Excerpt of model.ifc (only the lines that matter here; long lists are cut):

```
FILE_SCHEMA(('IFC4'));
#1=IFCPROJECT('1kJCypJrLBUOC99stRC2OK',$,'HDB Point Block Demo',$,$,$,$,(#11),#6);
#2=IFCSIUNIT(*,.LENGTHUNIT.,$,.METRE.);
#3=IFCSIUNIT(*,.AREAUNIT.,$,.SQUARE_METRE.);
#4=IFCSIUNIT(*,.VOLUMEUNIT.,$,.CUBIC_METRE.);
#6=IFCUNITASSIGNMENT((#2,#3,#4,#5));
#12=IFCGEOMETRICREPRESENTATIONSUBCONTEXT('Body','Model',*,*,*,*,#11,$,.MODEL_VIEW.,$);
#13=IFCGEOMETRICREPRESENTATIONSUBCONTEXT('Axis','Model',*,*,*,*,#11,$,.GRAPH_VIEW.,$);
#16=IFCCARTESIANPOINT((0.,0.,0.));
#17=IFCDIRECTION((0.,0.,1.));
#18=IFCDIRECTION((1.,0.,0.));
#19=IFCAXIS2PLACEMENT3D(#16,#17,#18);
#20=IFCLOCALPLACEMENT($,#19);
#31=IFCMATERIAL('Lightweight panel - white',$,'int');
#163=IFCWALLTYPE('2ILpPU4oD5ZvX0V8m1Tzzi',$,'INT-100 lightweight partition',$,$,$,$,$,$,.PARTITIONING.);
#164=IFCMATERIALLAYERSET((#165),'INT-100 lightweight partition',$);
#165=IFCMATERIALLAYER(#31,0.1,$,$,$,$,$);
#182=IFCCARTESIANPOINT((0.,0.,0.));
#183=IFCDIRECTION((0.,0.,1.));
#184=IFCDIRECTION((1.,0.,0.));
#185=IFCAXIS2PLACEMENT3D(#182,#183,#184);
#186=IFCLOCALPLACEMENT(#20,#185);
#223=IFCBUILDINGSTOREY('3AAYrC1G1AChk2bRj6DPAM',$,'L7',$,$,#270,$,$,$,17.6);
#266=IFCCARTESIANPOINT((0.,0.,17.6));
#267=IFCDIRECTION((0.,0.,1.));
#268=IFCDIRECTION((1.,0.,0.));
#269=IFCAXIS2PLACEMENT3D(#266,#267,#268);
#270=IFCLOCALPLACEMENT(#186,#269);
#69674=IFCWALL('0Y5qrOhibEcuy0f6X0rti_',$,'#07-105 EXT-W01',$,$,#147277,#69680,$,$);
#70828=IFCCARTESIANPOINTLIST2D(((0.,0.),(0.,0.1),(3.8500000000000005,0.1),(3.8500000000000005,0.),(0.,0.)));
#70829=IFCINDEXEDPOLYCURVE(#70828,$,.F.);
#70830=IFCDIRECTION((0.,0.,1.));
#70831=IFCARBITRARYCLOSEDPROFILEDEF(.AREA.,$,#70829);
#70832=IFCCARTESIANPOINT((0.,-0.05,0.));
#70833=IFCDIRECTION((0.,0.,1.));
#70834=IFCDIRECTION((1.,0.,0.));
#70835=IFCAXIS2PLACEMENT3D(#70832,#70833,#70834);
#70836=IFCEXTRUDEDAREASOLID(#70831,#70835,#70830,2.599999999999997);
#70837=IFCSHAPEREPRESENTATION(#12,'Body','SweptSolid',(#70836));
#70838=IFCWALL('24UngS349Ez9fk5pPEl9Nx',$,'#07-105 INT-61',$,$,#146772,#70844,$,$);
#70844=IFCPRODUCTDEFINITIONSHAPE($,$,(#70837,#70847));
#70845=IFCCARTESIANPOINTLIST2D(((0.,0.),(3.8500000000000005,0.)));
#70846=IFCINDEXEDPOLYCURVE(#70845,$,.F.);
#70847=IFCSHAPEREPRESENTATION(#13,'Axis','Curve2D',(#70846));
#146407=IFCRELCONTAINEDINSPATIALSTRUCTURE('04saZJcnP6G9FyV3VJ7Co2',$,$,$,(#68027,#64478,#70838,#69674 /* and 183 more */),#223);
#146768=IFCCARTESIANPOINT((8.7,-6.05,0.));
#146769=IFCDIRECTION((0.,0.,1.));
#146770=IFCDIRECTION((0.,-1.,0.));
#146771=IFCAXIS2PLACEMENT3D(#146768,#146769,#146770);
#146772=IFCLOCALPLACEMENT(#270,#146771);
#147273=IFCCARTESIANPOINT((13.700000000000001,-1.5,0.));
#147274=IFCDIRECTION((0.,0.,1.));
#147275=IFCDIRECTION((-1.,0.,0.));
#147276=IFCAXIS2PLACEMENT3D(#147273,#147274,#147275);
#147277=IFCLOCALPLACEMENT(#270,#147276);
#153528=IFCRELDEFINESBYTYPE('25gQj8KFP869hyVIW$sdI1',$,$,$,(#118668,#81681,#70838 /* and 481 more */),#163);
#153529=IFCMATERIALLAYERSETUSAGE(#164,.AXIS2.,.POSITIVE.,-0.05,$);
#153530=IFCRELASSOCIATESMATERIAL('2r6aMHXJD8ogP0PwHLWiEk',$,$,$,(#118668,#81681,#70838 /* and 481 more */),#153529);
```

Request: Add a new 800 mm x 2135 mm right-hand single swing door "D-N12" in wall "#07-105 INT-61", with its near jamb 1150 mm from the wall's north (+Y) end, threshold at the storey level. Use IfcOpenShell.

```python
import numpy as np
import ifcopenshell
import ifcopenshell.api.feature
import ifcopenshell.api.geometry
import ifcopenshell.api.root
import ifcopenshell.api.spatial
import ifcopenshell.geom
import ifcopenshell.util.element
import ifcopenshell.util.placement
import ifcopenshell.util.representation
import ifcopenshell.util.shape
import ifcopenshell.util.unit

model = ifcopenshell.open("model.ifc")
unit_scale = ifcopenshell.util.unit.calculate_unit_scale(model)
settings = ifcopenshell.geom.settings()


def volume(element):
    """Net volume in cubic metres, openings subtracted."""
    shape = ifcopenshell.geom.create_shape(settings, element)
    return ifcopenshell.util.shape.get_volume(shape.geometry)


wall = model.by_guid("24UngS349Ez9fk5pPEl9Nx")
storey = ifcopenshell.util.element.get_container(wall, ifc_class="IfcBuildingStorey")
context = ifcopenshell.util.representation.get_context(model, "Model", "Body", "MODEL_VIEW")
before = volume(wall)

width, height, from_end, sill = 0.8, 2.135, 1.15, 0.0  # metres

# The wall runs along its own X axis, and the end named is its -X end.
wall_shape = ifcopenshell.geom.create_shape(settings, wall)
x, y, z = ifcopenshell.util.shape.get_vertices(wall_shape.geometry).T
start = x.min() + from_end
face, thickness = float(y.min()), float(y.max() - y.min())
wall_matrix = ifcopenshell.util.placement.get_local_placement(wall.ObjectPlacement)
level = ifcopenshell.util.placement.get_local_placement(storey.ObjectPlacement)[2, 3]


def in_wall(x, y):
    """Placement at x, y metres in the wall's axes, at sill height."""
    matrix = wall_matrix.copy()
    matrix[:, 3] = wall_matrix @ np.array([x / unit_scale, y / unit_scale, 0.0, 1.0])
    matrix[2, 3] = level + sill / unit_scale
    return matrix


# Opening: a box that overshoots both wall faces by 50 mm.
opening = ifcopenshell.api.root.create_entity(model, ifc_class="IfcOpeningElement", predefined_type="OPENING")
box = ifcopenshell.api.geometry.add_wall_representation(
    model, context=context, length=width, height=height, thickness=thickness + 0.1
)
ifcopenshell.api.geometry.assign_representation(model, product=opening, representation=box)
ifcopenshell.api.geometry.edit_object_placement(model, product=opening, matrix=in_wall(start, face - 0.05), is_si=False)
ifcopenshell.api.feature.add_feature(model, feature=opening, element=wall)

door = ifcopenshell.api.root.create_entity(model, ifc_class="IfcDoor", name="D-N12", predefined_type="DOOR")
door.OverallWidth, door.OverallHeight = width / unit_scale, height / unit_scale
door.OperationType = "SINGLE_SWING_RIGHT"
body = ifcopenshell.api.geometry.add_door_representation(
    model,
    context=context,
    overall_width=door.OverallWidth,
    overall_height=door.OverallHeight,
    operation_type="SINGLE_SWING_RIGHT",
    lining_properties={"LiningDepth": thickness / unit_scale, "ThresholdDepth": thickness / unit_scale},
)
ifcopenshell.api.geometry.assign_representation(model, product=door, representation=body)
ifcopenshell.api.spatial.assign_container(model, products=[door], relating_structure=storey)
ifcopenshell.api.feature.add_filling(model, opening=opening, element=door)

# The lining spans the wall, so the door starts at the wall face.
ifcopenshell.api.geometry.edit_object_placement(model, product=door, matrix=in_wall(start, face), is_si=False)

after = volume(wall)

print(f"wall volume {before:.3f} -> {after:.3f} m3")

model.write("model-out.ifc")
```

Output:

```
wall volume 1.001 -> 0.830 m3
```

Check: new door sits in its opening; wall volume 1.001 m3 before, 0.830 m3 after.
